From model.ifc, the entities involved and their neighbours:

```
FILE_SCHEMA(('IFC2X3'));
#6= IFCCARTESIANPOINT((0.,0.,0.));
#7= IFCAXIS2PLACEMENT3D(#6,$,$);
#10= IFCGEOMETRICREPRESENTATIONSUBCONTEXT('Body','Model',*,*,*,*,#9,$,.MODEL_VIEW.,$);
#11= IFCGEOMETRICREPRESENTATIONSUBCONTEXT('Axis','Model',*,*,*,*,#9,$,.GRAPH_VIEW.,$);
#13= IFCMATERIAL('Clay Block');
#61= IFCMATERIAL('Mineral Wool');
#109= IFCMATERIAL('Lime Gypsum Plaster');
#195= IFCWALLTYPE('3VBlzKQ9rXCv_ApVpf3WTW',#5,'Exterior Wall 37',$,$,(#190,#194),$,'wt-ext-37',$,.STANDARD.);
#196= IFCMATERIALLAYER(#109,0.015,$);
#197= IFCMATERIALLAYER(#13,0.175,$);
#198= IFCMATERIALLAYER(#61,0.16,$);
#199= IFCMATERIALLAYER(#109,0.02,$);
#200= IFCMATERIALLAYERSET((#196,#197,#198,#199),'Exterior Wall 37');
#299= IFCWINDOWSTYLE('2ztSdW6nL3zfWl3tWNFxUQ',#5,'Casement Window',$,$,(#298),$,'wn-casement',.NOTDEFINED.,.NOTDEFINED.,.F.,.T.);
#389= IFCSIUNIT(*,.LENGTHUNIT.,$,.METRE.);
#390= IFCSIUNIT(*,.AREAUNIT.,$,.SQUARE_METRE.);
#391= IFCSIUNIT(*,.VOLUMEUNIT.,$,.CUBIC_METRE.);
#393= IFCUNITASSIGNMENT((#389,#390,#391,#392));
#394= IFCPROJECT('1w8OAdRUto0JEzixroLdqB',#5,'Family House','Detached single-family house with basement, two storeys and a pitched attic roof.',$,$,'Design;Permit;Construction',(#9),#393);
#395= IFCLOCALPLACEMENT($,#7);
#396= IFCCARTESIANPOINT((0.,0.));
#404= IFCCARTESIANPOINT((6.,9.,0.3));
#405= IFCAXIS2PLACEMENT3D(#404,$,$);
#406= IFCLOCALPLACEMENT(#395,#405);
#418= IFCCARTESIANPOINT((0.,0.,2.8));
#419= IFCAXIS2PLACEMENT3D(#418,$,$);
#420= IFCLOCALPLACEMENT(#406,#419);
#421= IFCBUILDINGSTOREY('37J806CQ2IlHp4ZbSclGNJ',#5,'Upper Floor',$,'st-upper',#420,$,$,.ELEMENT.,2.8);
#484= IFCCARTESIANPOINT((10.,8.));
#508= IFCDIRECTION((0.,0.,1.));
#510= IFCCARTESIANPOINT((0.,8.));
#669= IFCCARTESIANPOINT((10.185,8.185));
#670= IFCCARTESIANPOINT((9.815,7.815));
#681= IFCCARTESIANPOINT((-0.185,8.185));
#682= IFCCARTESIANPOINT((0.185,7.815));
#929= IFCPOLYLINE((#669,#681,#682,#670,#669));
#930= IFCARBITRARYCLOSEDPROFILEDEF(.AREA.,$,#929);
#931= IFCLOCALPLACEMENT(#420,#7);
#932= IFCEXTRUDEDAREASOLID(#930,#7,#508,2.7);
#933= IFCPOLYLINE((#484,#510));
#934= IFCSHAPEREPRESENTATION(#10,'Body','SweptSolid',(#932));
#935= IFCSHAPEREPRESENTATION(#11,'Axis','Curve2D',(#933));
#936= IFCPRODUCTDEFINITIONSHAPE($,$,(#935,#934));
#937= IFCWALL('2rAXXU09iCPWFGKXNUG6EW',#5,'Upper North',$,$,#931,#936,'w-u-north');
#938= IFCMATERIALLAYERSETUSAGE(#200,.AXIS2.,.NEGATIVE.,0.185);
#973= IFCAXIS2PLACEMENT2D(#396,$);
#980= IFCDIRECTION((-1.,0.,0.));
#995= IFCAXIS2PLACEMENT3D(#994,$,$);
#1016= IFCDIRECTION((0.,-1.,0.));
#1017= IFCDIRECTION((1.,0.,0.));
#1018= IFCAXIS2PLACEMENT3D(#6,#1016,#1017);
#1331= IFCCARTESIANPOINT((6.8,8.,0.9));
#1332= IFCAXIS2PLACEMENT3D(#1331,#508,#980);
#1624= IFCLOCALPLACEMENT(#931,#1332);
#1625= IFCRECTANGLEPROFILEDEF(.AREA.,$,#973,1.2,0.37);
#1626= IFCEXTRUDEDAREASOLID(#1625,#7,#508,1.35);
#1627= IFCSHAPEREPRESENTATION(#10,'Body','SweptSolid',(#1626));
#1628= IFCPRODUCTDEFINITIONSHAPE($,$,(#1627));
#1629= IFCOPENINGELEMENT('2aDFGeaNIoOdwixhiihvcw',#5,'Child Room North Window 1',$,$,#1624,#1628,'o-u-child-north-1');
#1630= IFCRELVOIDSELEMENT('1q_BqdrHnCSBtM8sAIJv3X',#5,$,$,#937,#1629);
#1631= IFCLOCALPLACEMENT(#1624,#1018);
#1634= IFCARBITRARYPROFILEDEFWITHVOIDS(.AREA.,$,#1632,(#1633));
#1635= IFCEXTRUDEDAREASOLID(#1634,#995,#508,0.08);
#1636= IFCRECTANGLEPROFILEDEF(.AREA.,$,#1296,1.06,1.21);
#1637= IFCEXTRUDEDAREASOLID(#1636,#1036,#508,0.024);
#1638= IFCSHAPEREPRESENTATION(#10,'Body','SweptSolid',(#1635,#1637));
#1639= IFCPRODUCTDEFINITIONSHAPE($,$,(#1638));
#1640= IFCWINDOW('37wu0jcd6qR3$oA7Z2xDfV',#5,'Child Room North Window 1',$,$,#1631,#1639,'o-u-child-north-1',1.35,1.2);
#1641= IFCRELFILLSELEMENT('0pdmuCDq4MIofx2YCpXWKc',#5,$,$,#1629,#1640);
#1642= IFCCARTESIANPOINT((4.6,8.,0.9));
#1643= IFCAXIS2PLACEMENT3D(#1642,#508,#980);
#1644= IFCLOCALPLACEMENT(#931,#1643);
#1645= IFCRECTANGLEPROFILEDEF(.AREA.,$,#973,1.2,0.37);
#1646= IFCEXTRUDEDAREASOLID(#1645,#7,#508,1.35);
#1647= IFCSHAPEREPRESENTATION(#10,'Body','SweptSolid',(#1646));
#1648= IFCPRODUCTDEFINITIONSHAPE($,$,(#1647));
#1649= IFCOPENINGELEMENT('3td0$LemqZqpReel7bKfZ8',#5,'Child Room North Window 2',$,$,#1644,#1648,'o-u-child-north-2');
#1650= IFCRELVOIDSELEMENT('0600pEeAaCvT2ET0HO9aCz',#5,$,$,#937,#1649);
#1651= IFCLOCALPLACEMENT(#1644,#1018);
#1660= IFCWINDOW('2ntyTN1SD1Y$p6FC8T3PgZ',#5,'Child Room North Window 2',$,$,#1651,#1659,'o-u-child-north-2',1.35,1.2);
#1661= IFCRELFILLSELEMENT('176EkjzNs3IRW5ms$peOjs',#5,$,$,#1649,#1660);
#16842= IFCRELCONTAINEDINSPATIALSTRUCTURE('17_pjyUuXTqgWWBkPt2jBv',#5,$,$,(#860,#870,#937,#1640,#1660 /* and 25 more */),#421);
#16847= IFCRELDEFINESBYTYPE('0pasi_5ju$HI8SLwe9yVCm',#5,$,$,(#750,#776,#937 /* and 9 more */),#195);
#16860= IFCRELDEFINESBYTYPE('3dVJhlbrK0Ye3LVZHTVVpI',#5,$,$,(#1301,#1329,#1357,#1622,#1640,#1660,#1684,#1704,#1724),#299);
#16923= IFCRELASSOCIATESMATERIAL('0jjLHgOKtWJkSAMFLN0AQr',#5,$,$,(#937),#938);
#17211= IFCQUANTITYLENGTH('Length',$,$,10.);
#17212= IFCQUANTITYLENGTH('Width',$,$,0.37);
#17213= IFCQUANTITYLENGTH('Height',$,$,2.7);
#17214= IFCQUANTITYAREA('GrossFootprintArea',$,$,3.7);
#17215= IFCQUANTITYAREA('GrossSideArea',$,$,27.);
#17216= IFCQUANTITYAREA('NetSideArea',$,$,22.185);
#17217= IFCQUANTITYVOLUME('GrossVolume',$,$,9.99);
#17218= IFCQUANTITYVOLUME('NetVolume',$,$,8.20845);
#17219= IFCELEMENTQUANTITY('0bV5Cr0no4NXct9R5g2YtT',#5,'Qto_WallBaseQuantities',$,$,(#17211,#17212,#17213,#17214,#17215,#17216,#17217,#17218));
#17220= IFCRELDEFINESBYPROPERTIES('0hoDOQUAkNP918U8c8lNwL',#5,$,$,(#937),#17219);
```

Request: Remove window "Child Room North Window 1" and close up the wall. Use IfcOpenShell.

```python
import ifcopenshell
import ifcopenshell.api.feature
import ifcopenshell.api.pset
import ifcopenshell.api.root
import ifcopenshell.geom
import ifcopenshell.util.element
import ifcopenshell.util.shape
import ifcopenshell.util.unit

model = ifcopenshell.open("model.ifc")
area_scale = ifcopenshell.util.unit.calculate_unit_scale(model, "AREAUNIT")
volume_scale = ifcopenshell.util.unit.calculate_unit_scale(model, "VOLUMEUNIT")
settings = ifcopenshell.geom.settings()


def volume(element):
    """Net volume in cubic metres, openings subtracted."""
    shape = ifcopenshell.geom.create_shape(settings, element)
    return ifcopenshell.util.shape.get_volume(shape.geometry)


window = model.by_id(1640)
opening = window.FillsVoids[0].RelatingOpeningElement
wall = opening.VoidsElements[0].RelatingBuildingElement
before = volume(wall)

ifcopenshell.api.root.remove_product(model, product=window)
ifcopenshell.api.feature.remove_feature(model, feature=opening)

after = volume(wall)
thickness = 0.37  # wall thickness in metres

# Update the wall's stored quantities.
qto = model.by_id(ifcopenshell.util.element.get_pset(wall, "Qto_WallBaseQuantities", should_inherit=False)["id"])
ifcopenshell.api.pset.edit_qto(model, qto=qto, properties={
    "NetSideArea": after / thickness / area_scale,
    "NetVolume": after / volume_scale,
})

print(f"wall volume {before:.3f} -> {after:.3f} m3")

model.write("model_v2.ifc")
```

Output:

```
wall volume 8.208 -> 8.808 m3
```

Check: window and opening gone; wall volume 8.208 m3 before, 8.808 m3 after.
